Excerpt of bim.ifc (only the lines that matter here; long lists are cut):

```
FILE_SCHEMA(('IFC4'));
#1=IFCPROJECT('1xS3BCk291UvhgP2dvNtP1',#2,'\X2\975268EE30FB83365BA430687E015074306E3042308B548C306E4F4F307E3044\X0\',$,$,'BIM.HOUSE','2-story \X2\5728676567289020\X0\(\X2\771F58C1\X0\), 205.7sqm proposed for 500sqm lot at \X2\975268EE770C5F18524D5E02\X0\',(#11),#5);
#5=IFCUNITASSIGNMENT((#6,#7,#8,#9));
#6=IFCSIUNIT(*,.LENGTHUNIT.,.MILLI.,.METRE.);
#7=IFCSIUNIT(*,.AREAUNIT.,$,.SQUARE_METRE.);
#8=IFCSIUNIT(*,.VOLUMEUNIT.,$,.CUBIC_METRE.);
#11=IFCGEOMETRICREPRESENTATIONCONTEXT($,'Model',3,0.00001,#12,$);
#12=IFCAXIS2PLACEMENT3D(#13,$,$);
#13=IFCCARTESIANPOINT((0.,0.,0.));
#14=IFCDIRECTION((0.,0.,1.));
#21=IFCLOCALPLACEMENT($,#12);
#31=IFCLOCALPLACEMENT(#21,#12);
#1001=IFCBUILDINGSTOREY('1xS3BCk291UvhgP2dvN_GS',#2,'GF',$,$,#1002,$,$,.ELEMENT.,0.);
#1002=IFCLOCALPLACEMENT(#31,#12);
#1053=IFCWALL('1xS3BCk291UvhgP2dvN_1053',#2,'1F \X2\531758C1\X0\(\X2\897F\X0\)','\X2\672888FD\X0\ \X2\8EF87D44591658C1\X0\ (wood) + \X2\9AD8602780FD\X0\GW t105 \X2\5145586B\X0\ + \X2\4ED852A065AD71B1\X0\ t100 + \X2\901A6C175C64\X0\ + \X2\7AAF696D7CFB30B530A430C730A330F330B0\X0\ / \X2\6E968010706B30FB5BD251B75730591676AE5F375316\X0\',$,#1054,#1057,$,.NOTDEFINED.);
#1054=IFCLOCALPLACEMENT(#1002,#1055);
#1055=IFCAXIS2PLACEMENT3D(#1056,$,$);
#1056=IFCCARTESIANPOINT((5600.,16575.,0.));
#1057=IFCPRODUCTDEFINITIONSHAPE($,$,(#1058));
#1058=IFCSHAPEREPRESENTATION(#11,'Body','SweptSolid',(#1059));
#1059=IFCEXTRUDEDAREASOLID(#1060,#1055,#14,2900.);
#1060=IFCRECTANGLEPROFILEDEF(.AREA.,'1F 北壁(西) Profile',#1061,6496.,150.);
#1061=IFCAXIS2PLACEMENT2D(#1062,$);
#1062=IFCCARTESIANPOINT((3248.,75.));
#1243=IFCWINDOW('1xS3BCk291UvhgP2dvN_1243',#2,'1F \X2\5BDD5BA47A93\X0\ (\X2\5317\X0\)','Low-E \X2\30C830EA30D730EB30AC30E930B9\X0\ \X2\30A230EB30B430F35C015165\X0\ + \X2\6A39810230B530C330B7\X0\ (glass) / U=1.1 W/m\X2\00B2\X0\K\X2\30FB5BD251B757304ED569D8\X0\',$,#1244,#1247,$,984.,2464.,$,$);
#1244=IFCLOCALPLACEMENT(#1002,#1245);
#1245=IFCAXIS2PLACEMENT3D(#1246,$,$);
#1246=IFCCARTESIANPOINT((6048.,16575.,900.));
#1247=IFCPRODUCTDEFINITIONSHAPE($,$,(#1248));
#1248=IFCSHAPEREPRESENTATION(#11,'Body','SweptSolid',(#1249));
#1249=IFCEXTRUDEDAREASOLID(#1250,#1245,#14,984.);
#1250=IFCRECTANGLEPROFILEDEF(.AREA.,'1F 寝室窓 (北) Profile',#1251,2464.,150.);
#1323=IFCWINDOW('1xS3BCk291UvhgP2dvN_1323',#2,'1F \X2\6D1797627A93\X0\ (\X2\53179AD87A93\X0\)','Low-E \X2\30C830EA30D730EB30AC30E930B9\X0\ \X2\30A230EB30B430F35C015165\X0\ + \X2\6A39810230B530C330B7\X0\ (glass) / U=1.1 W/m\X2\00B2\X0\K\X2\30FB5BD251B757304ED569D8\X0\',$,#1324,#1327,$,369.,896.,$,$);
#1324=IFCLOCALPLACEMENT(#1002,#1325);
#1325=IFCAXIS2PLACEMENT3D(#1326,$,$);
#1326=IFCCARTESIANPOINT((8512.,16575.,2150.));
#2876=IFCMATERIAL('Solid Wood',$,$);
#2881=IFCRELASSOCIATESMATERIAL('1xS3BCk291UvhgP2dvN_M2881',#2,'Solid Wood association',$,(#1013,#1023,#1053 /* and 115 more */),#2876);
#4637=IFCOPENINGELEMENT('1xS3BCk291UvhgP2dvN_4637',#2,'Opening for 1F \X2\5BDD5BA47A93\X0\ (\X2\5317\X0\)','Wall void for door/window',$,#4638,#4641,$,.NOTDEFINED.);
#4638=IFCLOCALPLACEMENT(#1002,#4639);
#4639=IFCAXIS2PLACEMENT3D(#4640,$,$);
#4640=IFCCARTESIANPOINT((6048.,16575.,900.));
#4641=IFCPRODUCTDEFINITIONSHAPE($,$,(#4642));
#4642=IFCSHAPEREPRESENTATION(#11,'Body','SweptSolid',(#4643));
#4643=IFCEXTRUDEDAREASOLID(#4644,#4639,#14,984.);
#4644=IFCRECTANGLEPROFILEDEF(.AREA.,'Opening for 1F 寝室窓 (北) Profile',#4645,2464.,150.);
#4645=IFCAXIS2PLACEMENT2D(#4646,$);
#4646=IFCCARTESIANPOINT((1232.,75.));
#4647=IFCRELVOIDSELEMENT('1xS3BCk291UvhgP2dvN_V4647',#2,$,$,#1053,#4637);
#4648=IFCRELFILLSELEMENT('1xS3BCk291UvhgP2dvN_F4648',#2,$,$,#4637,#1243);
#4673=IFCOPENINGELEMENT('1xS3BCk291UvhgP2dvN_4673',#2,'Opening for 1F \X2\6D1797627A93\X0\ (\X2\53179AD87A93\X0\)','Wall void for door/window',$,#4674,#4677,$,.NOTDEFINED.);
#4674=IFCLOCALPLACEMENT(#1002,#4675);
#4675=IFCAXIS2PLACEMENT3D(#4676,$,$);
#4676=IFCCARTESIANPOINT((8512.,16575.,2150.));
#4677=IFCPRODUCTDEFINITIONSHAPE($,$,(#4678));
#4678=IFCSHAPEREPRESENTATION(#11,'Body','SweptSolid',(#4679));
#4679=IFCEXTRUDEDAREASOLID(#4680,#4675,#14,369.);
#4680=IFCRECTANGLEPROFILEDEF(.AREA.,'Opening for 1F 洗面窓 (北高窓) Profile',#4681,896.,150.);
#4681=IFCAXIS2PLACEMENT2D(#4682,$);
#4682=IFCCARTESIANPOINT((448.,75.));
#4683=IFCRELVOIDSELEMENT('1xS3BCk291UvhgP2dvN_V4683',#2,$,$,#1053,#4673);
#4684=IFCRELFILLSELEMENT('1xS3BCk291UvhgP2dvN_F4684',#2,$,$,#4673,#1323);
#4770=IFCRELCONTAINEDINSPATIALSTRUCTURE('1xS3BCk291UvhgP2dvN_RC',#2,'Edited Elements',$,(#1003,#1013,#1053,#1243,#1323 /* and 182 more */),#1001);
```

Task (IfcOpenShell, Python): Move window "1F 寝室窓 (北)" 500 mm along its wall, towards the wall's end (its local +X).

```python
import ifcopenshell
import ifcopenshell.api.geometry
import ifcopenshell.util.placement
import ifcopenshell.util.unit

model = ifcopenshell.open("bim.ifc")
unit_scale = ifcopenshell.util.unit.calculate_unit_scale(model)

window = model.by_guid("1xS3BCk291UvhgP2dvN_1243")
opening = window.FillsVoids[0].RelatingOpeningElement
wall = opening.VoidsElements[0].RelatingBuildingElement

wall_matrix = ifcopenshell.util.placement.get_local_placement(wall.ObjectPlacement)
shift = wall_matrix[:3, 0] * 0.5 / unit_scale
before = ifcopenshell.util.placement.get_local_placement(window.ObjectPlacement)[:3, 3].copy()

# The window is not placed relative to its opening, so move both.
for product in (opening, window):
    matrix = ifcopenshell.util.placement.get_local_placement(product.ObjectPlacement)
    matrix[:3, 3] += shift
    ifcopenshell.api.geometry.edit_object_placement(model, product=product, matrix=matrix, is_si=False)

after = ifcopenshell.util.placement.get_local_placement(window.ObjectPlacement)[:3, 3]
print("window moved by", (after - before).round(3) + 0.0)

model.write("bim_updated.ifc")
```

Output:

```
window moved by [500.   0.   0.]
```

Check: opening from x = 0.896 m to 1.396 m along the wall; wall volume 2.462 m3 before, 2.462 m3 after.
